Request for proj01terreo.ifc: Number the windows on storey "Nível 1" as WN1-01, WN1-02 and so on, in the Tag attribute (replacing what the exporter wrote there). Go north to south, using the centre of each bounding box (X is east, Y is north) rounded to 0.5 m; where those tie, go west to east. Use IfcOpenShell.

First a look at what the model holds.

```python
import ifcopenshell
import ifcopenshell.util.element
import ifcopenshell.util.placement

model = ifcopenshell.open("proj01terreo.ifc")
print(model.schema)
storey = next(s for s in model.by_type("IfcBuildingStorey") if s.Name == "Nível 1")
windows = [e for e in ifcopenshell.util.element.get_decomposition(storey) if e.is_a("IfcWindow")]
for e in sorted(windows, key=lambda e: e.id()):
    origin = ifcopenshell.util.placement.get_local_placement(e.ObjectPlacement)[:3, 3]
    print(e.id(), e.Tag, e.Name, origin.round(2) + 0.0, sep=" | ")
```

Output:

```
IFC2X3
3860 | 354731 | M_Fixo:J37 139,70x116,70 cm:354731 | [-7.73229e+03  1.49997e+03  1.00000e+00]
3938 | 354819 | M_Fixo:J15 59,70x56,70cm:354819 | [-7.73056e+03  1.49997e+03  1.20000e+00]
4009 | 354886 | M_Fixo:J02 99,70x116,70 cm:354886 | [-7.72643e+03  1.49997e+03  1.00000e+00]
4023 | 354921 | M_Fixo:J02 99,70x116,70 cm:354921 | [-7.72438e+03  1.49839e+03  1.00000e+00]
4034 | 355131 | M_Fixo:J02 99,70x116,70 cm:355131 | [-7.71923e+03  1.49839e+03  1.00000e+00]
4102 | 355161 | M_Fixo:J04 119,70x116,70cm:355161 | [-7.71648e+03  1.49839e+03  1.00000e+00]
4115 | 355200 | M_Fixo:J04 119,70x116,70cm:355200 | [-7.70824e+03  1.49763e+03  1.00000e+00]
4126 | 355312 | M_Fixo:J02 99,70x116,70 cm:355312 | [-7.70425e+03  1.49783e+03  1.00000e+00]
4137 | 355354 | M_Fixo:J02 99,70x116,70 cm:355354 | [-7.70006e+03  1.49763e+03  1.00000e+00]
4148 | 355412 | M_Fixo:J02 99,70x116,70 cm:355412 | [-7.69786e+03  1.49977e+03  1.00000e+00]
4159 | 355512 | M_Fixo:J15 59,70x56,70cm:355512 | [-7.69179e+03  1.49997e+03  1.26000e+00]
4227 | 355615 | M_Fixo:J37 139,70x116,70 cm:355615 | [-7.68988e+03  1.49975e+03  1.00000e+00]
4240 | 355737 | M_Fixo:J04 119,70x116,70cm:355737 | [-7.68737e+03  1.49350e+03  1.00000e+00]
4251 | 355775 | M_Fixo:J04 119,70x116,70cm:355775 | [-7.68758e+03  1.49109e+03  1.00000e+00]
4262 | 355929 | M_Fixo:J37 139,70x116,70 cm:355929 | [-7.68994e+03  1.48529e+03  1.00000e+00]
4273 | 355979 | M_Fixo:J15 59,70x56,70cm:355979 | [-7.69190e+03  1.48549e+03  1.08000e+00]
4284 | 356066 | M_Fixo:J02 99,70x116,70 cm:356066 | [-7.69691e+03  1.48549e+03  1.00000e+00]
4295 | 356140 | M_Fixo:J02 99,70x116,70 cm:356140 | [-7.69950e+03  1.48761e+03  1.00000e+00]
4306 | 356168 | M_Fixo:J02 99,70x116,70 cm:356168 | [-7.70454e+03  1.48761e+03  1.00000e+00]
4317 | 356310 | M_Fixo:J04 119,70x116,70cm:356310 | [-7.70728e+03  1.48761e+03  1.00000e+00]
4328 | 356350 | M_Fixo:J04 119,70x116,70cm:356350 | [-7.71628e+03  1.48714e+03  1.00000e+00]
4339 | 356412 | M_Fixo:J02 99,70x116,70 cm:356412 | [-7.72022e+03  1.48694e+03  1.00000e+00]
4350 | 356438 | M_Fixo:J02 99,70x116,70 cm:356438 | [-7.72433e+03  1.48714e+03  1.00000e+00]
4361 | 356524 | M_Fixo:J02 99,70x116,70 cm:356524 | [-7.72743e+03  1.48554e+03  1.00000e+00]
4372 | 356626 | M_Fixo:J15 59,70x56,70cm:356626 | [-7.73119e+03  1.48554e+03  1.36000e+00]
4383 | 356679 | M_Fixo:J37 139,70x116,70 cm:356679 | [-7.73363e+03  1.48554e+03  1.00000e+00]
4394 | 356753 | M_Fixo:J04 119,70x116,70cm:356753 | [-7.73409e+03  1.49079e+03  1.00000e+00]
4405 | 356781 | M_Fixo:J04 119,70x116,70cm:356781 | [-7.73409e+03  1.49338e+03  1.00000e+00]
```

```python
import ifcopenshell
import ifcopenshell.geom
import ifcopenshell.util.element
import ifcopenshell.util.shape

model = ifcopenshell.open("proj01terreo.ifc")
settings = ifcopenshell.geom.settings()
settings.set("use-world-coords", True)


def centre(element):
    shape = ifcopenshell.geom.create_shape(settings, element)
    return ifcopenshell.util.shape.get_bbox_centroid(shape.geometry)


storey = next(s for s in model.by_type("IfcBuildingStorey") if s.Name == "Nível 1")
windows = [e for e in ifcopenshell.util.element.get_decomposition(storey) if e.is_a("IfcWindow")]

# Insertion points can sit at a corner or the storey origin, so sort by the geometry (in metres).
centres = {e: centre(e) for e in windows}
windows.sort(key=lambda e: (-round(centres[e][1] / 0.5), centres[e][0]))

for i, e in enumerate(windows, start=1):
    number = f"WN1-{i:02d}"
    e.Tag = number
    print(e.id(), number)

model.write("proj01terreo_updated.ifc")
```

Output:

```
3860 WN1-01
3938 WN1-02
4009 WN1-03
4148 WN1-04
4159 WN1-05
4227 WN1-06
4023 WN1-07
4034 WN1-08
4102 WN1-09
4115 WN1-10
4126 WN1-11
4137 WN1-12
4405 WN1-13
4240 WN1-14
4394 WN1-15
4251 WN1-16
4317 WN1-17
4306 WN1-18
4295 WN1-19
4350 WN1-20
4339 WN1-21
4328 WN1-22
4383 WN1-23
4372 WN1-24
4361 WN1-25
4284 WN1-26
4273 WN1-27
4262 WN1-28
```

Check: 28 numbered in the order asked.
